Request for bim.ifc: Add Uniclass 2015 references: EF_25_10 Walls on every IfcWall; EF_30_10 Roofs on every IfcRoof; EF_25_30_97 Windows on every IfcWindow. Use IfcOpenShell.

First a look at what the model holds.

```python
import ifcopenshell

model = ifcopenshell.open("bim.ifc")
print(model.schema)
print("classifications:", [c.Name for c in model.by_type("IfcClassification")])
for ifc_class in ("IfcDoor", "IfcRoof", "IfcStair", "IfcWall", "IfcWindow"):
    print(ifc_class, len(model.by_type(ifc_class)))
```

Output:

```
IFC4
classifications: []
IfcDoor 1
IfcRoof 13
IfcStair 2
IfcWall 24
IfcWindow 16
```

```python
import ifcopenshell
import ifcopenshell.api.classification

model = ifcopenshell.open("bim.ifc")

system = ifcopenshell.api.classification.add_classification(model, classification="Uniclass 2015")

codes = {
    "IfcWall": ("EF_25_10", "Walls"),
    "IfcRoof": ("EF_30_10", "Roofs"),
    "IfcWindow": ("EF_25_30_97", "Windows"),
}
for ifc_class, (code, name) in codes.items():
    products = model.by_type(ifc_class)
    ifcopenshell.api.classification.add_reference(
        model, products=products, classification=system, identification=code, name=name
    )
    print(code, len(products))

model.write("bim_v2.ifc")
```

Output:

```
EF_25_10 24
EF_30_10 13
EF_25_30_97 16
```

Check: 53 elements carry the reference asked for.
